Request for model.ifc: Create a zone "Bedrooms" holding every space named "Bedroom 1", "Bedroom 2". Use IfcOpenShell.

First a look at what the model holds.

```python
import ifcopenshell

model = ifcopenshell.open("model.ifc")
print(model.schema)
seen = {}
for space in model.by_type("IfcSpace"):
    seen[space.Name] = seen.get(space.Name, 0) + 1
for name, count in sorted(seen.items(), key=str):
    print(count, "x", name)
print("zones:", [z.Name for z in model.by_type("IfcZone")][:20])
```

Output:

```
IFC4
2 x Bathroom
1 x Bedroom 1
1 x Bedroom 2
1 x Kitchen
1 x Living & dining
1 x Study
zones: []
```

```python
import ifcopenshell
import ifcopenshell.api.group
import ifcopenshell.api.root

model = ifcopenshell.open("model.ifc")

names = {"Bedroom 1", "Bedroom 2"}
spaces = [s for s in model.by_type("IfcSpace") if s.Name in names]

zone = ifcopenshell.api.root.create_entity(model, ifc_class="IfcZone", name="Bedrooms")
ifcopenshell.api.group.assign_group(model, products=spaces, group=zone)
print(len(spaces), "spaces in", zone.Name)

model.write("model_rev.ifc")
```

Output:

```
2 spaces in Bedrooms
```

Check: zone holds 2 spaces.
